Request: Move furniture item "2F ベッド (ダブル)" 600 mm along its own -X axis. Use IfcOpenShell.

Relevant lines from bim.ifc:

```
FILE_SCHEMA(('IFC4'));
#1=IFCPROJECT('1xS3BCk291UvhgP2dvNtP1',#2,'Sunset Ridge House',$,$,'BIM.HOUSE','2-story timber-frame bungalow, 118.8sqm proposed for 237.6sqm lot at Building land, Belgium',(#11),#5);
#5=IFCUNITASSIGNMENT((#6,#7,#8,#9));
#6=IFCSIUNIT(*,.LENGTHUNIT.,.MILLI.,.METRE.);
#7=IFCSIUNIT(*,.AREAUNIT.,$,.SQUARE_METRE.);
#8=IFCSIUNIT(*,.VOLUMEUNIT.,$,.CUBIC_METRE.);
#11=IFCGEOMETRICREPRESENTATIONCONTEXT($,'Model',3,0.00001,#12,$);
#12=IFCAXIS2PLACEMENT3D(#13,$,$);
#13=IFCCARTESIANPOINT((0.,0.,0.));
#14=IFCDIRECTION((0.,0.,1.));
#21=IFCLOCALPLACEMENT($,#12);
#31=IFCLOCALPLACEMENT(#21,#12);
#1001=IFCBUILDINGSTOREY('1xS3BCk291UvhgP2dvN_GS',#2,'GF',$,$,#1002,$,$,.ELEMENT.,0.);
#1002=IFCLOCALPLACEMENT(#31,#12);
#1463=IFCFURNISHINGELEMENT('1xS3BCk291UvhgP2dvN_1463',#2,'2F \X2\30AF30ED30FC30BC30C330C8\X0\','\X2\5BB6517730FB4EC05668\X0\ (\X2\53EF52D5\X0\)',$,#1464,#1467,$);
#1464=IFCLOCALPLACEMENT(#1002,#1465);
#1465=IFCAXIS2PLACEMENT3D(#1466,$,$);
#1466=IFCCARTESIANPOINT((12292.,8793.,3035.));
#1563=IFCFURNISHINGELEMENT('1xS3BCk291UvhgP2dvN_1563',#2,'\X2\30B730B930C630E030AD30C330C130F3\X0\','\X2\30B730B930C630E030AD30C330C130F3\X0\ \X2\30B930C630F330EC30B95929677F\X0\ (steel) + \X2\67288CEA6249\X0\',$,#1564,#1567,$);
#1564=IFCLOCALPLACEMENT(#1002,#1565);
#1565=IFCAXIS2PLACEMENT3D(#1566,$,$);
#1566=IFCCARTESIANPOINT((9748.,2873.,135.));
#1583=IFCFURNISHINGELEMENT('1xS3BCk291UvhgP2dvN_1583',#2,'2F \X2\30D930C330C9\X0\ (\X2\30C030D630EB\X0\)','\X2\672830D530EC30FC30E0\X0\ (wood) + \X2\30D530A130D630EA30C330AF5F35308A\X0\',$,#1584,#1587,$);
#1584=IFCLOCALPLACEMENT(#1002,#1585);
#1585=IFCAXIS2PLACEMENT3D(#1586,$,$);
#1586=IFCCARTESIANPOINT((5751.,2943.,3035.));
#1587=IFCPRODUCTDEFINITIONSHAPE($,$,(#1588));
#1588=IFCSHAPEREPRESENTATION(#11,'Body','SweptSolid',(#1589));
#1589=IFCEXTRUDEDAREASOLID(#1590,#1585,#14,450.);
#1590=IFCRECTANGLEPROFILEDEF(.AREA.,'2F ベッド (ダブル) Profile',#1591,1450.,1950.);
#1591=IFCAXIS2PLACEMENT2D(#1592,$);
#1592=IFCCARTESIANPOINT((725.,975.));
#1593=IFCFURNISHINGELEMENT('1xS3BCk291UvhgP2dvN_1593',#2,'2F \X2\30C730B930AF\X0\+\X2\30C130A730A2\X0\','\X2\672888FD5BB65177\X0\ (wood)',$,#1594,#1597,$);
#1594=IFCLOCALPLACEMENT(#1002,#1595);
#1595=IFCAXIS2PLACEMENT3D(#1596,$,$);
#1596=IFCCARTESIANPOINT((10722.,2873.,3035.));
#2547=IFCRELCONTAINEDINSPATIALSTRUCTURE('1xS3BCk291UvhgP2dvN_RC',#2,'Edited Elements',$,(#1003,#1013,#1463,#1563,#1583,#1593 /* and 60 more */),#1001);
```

```python
import ifcopenshell
import ifcopenshell.api.geometry
import ifcopenshell.util.placement

model = ifcopenshell.open("bim.ifc")

item = model.by_guid("1xS3BCk291UvhgP2dvN_1583")
matrix = ifcopenshell.util.placement.get_local_placement(item.ObjectPlacement)
matrix[:3, 3] -= matrix[:3, 0] * 600.0
ifcopenshell.api.geometry.edit_object_placement(model, product=item, matrix=matrix, is_si=False)

print(ifcopenshell.util.placement.get_local_placement(item.ObjectPlacement).round(3) + 0.0)

model.write("bim-out.ifc")
```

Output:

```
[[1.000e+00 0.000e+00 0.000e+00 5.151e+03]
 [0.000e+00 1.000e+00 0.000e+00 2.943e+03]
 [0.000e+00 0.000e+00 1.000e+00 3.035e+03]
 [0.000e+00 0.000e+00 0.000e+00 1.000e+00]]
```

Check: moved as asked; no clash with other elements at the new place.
